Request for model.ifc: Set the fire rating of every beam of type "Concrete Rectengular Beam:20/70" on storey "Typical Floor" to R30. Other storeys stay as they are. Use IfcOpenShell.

First a look at what the model holds.

```python
import ifcopenshell
import ifcopenshell.util.element

model = ifcopenshell.open("model.ifc")
print(model.schema)
storey = next(s for s in model.by_type("IfcBuildingStorey") if s.Name == "Typical Floor")
beams = [e for e in ifcopenshell.util.element.get_decomposition(storey) if e.is_a("IfcBeam")]
seen = {}
for e in beams:
    element_type = ifcopenshell.util.element.get_type(e)
    key = (element_type.Name if element_type != e and element_type else None, ifcopenshell.util.element.get_pset(e, "Pset_BeamCommon", "FireRating"))
    seen[key] = seen.get(key, 0) + 1
for (name, value), count in sorted(seen.items(), key=str):
    print(count, "x", name, "|", value)
```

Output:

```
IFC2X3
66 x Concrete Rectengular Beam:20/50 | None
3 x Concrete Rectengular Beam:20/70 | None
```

```python
import ifcopenshell
import ifcopenshell.api.pset
import ifcopenshell.util.element

model = ifcopenshell.open("model.ifc")

storey = next(s for s in model.by_type("IfcBuildingStorey") if s.Name == "Typical Floor")
beams = [e for e in ifcopenshell.util.element.get_decomposition(storey) if e.is_a("IfcBeam")]

count = 0
for e in beams:
    element_type = ifcopenshell.util.element.get_type(e)
    if element_type in (None, e) or element_type.Name != "Concrete Rectengular Beam:20/70":
        continue
    # add_pset returns the element's existing set when there is one.
    pset = ifcopenshell.api.pset.add_pset(model, product=e, name="Pset_BeamCommon")
    ifcopenshell.api.pset.edit_pset(model, pset=pset, properties={"FireRating": "R30"})
    count += 1

print(count, "beams updated")

model.write("model-out.ifc")
```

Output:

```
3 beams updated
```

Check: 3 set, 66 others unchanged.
